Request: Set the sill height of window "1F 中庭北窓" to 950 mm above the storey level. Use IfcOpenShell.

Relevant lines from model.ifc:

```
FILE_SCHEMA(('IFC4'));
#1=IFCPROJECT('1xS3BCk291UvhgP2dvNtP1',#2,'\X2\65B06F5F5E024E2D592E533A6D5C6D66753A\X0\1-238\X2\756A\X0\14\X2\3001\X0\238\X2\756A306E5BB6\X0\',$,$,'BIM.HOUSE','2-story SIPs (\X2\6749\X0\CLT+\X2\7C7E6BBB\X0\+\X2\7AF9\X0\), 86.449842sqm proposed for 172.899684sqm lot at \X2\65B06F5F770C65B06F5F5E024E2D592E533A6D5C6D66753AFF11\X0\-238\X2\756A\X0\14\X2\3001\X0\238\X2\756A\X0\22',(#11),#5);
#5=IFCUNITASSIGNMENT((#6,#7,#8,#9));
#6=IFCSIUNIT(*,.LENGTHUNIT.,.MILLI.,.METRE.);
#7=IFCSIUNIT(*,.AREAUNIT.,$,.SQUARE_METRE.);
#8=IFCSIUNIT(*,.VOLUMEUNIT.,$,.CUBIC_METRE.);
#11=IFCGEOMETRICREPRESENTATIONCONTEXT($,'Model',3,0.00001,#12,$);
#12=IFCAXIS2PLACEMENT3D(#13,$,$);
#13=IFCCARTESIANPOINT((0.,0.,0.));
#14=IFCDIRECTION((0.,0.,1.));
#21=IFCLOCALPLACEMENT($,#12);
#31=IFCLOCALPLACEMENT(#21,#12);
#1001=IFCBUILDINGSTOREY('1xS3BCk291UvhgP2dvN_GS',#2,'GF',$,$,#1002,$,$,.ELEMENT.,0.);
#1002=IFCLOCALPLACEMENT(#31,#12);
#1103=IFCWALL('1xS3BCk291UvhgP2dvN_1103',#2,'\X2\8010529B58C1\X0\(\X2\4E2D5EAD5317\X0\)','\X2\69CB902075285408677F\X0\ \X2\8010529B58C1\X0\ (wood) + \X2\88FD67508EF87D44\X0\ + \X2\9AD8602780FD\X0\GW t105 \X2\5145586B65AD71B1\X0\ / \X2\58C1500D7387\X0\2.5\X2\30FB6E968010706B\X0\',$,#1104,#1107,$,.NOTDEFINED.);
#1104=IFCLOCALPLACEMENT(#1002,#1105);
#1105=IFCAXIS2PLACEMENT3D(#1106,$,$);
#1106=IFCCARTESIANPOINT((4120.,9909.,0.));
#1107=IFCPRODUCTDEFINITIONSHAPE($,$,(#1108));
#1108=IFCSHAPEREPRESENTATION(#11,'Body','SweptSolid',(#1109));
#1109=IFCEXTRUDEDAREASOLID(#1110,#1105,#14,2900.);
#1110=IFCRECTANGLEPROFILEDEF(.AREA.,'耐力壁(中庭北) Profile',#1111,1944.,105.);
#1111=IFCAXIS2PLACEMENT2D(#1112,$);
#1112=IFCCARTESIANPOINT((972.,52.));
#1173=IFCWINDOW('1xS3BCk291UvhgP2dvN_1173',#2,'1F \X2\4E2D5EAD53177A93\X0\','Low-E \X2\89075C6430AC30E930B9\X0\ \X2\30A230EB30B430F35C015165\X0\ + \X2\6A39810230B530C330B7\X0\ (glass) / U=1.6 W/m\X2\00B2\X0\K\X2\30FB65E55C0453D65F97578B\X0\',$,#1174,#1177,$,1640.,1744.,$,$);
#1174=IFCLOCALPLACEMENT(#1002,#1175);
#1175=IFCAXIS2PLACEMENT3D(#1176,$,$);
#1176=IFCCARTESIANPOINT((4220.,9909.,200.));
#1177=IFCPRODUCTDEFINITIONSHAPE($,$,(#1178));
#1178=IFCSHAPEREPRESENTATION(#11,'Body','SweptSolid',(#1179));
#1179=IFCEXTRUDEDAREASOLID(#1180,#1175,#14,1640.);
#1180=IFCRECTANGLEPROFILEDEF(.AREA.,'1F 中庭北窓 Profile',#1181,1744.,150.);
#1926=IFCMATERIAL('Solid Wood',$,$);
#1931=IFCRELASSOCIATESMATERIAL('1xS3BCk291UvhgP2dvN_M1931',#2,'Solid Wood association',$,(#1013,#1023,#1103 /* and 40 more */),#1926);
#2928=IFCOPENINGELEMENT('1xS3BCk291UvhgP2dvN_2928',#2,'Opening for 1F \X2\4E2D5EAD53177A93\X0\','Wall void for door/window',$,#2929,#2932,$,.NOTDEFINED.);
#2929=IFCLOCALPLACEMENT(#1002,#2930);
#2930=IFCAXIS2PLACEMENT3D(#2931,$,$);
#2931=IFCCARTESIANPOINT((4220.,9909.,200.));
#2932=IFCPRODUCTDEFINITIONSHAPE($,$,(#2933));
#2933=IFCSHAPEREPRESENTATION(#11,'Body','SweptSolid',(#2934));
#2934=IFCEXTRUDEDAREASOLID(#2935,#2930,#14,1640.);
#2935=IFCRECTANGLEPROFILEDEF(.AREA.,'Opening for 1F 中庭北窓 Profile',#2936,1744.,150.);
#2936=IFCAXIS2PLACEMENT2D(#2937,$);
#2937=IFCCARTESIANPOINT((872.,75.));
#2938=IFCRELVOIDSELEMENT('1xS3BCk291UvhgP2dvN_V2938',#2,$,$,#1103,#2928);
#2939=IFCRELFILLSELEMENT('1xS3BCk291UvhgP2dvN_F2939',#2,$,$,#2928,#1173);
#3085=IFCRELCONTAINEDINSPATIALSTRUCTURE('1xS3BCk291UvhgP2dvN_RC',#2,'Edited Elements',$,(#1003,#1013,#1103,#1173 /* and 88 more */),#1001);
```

```python
import numpy as np
import ifcopenshell
import ifcopenshell.api.geometry
import ifcopenshell.geom
import ifcopenshell.util.element
import ifcopenshell.util.placement
import ifcopenshell.util.shape
import ifcopenshell.util.unit

model = ifcopenshell.open("model.ifc")
unit_scale = ifcopenshell.util.unit.calculate_unit_scale(model)

window = model.by_guid("1xS3BCk291UvhgP2dvN_1173")
opening = window.FillsVoids[0].RelatingOpeningElement
storey = ifcopenshell.util.element.get_container(window, ifc_class="IfcBuildingStorey")
level = ifcopenshell.util.placement.get_local_placement(storey.ObjectPlacement)[2, 3]

# The opening's origin need not be at the sill, so measure its lowest point.
shape = ifcopenshell.geom.create_shape(ifcopenshell.geom.settings(), opening)
bottom = ifcopenshell.util.shape.get_shape_bottom_elevation(shape, shape.geometry) / unit_scale
dz = level + 0.95 / unit_scale - bottom

shift = np.array([0.0, 0.0, dz])
# The window is not placed relative to its opening, so move both.
for product in (opening, window):
    matrix = ifcopenshell.util.placement.get_local_placement(product.ObjectPlacement)
    matrix[:3, 3] += shift
    ifcopenshell.api.geometry.edit_object_placement(model, product=product, matrix=matrix, is_si=False)

print(f"moved by {dz * unit_scale:+.3f} m")

model.write("model-out.ifc")
```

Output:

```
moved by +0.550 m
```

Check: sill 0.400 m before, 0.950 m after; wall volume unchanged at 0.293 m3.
